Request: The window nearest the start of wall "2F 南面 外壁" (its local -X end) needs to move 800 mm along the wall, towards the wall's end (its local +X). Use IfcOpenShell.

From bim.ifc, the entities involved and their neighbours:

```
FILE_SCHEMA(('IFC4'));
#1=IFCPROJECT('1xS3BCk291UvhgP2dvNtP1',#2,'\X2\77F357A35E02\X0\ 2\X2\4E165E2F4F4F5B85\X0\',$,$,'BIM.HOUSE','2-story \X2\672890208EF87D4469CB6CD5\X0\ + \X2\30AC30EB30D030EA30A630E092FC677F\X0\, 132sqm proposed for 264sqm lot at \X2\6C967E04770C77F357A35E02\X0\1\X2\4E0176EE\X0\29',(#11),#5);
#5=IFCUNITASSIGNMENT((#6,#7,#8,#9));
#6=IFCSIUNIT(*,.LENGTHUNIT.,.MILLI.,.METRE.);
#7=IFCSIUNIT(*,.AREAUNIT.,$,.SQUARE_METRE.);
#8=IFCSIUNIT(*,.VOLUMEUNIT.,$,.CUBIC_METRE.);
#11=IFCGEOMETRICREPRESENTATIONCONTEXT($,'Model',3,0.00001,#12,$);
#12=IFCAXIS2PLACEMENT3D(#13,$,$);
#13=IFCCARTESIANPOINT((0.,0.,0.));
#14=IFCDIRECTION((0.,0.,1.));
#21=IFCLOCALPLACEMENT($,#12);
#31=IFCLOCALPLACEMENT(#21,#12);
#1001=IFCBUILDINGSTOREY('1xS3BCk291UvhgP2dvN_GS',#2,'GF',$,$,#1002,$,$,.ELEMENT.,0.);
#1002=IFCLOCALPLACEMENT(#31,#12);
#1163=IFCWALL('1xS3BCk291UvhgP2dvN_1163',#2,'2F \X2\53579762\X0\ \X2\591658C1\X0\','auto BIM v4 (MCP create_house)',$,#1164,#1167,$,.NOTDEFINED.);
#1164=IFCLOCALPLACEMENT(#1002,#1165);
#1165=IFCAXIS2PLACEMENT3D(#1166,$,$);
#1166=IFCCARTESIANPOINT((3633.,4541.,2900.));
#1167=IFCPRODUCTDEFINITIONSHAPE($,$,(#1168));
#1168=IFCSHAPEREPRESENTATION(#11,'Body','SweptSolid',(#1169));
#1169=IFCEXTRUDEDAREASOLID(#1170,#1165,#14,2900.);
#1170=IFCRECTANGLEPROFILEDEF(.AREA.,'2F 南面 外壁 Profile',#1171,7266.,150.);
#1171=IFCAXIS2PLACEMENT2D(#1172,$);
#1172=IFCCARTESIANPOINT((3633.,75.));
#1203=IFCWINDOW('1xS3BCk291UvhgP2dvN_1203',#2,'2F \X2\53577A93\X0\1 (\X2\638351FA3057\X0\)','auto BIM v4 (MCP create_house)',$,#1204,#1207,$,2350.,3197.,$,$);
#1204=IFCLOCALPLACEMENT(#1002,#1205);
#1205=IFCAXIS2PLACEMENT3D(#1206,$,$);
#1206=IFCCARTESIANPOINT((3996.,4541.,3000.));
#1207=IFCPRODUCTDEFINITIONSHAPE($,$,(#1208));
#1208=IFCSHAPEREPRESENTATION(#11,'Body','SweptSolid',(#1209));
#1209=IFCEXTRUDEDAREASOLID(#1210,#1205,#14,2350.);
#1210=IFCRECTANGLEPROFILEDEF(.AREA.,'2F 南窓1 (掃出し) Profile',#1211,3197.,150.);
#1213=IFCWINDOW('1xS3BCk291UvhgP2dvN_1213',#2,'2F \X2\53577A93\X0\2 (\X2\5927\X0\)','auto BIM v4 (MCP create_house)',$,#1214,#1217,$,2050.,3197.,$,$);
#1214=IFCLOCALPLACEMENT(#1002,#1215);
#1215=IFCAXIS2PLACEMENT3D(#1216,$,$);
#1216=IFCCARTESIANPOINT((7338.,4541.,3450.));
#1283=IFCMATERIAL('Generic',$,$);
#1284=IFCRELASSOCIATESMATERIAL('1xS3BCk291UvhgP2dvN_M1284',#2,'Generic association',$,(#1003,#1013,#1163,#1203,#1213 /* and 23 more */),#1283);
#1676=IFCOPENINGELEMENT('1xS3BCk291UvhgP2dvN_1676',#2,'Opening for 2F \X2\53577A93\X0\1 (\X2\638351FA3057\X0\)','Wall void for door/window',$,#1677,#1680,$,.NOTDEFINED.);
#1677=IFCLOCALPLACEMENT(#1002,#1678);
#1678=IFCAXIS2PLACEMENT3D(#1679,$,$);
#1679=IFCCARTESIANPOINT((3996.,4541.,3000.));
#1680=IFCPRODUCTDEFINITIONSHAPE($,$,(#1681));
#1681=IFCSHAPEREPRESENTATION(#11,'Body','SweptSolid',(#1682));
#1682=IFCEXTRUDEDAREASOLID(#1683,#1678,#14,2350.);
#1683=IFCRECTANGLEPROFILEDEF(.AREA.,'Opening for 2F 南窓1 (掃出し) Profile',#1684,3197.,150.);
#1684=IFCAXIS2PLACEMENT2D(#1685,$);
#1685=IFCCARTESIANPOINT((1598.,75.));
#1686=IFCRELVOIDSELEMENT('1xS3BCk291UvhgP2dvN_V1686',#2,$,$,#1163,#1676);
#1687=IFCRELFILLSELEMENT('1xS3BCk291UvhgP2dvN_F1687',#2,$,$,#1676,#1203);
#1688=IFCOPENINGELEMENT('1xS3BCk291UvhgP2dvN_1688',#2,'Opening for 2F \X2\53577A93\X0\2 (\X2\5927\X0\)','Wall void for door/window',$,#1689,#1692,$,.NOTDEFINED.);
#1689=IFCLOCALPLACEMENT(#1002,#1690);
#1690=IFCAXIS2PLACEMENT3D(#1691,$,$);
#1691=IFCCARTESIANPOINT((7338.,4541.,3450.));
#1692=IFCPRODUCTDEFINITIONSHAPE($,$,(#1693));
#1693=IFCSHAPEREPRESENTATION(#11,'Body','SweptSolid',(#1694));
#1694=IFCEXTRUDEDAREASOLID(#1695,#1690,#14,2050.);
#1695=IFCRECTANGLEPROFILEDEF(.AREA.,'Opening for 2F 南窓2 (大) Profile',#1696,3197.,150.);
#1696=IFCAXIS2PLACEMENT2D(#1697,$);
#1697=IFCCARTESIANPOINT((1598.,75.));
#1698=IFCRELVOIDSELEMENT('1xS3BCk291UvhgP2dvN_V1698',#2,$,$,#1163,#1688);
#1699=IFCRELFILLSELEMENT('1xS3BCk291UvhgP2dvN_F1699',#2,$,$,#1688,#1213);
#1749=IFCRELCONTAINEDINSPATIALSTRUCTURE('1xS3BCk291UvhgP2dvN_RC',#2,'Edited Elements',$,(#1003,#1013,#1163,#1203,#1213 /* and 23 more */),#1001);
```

```python
import ifcopenshell
import ifcopenshell.api.geometry
import ifcopenshell.util.placement
import ifcopenshell.util.unit

model = ifcopenshell.open("bim.ifc")
unit_scale = ifcopenshell.util.unit.calculate_unit_scale(model)

window = model.by_guid("1xS3BCk291UvhgP2dvN_1203")
opening = window.FillsVoids[0].RelatingOpeningElement
wall = opening.VoidsElements[0].RelatingBuildingElement

wall_matrix = ifcopenshell.util.placement.get_local_placement(wall.ObjectPlacement)
shift = wall_matrix[:3, 0] * 0.8 / unit_scale
before = ifcopenshell.util.placement.get_local_placement(window.ObjectPlacement)[:3, 3].copy()

# The window is not placed relative to its opening, so move both.
for product in (opening, window):
    matrix = ifcopenshell.util.placement.get_local_placement(product.ObjectPlacement)
    matrix[:3, 3] += shift
    ifcopenshell.api.geometry.edit_object_placement(model, product=product, matrix=matrix, is_si=False)

after = ifcopenshell.util.placement.get_local_placement(window.ObjectPlacement)[:3, 3]
print("window moved by", (after - before).round(3) + 0.0)

model.write("bim_updated.ifc")
```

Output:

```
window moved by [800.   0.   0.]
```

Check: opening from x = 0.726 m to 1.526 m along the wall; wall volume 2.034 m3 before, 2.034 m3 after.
